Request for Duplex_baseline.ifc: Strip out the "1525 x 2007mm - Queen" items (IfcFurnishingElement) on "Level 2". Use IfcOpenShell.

First a look at what the model holds.

```python
import ifcopenshell
import ifcopenshell.util.element

model = ifcopenshell.open("Duplex_baseline.ifc")
print(model.schema)
storey = next(s for s in model.by_type("IfcBuildingStorey") if s.Name == "Level 2")
furniture = [e for e in ifcopenshell.util.element.get_decomposition(storey) if e.is_a("IfcFurnishingElement")]
seen = {}
for e in furniture:
    element_type = ifcopenshell.util.element.get_type(e)
    name = element_type.Name if element_type not in (None, e) else None
    seen[name] = seen.get(name, 0) + 1
for name, count in sorted(seen.items(), key=str):
    print(count, "x", name)
```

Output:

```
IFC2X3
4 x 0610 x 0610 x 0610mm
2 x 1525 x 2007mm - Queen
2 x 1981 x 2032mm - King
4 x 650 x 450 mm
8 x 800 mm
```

```python
import ifcopenshell
import ifcopenshell.api.root
import ifcopenshell.util.element

model = ifcopenshell.open("Duplex_baseline.ifc")

storey = next(s for s in model.by_type("IfcBuildingStorey") if s.Name == "Level 2")
furniture = [e for e in ifcopenshell.util.element.get_decomposition(storey) if e.is_a("IfcFurnishingElement")]
targets = [e for e in furniture if (t := ifcopenshell.util.element.get_type(e)) not in (None, e) and t.Name == "1525 x 2007mm - Queen"]

for e in targets:
    ifcopenshell.api.root.remove_product(model, product=e)
print(len(targets), "removed")

model.write("Duplex_baseline_v2.ifc")
```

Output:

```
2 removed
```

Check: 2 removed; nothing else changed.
